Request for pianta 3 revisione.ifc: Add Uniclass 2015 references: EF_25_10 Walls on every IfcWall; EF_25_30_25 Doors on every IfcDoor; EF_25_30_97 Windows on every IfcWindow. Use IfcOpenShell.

First a look at what the model holds.

```python
import ifcopenshell

model = ifcopenshell.open("pianta 3 revisione.ifc")
print(model.schema)
print("classifications:", [c.Name for c in model.by_type("IfcClassification")])
for ifc_class in ("IfcDoor", "IfcRoof", "IfcStair", "IfcWall", "IfcWindow"):
    print(ifc_class, len(model.by_type(ifc_class)))
```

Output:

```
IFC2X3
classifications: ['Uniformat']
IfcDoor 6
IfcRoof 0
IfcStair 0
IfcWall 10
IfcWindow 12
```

```python
import ifcopenshell
import ifcopenshell.api.classification

model = ifcopenshell.open("pianta 3 revisione.ifc")

# IFC2X3 requires Source and Edition and has no link from the project to the system.
system = model.create_entity("IfcClassification", Source="NBS", Edition="2015", Name="Uniclass 2015")

codes = {
    "IfcWall": ("EF_25_10", "Walls"),
    "IfcDoor": ("EF_25_30_25", "Doors"),
    "IfcWindow": ("EF_25_30_97", "Windows"),
}
for ifc_class, (code, name) in codes.items():
    products = model.by_type(ifc_class)
    ifcopenshell.api.classification.add_reference(
        model, products=products, classification=system, identification=code, name=name
    )
    print(code, len(products))

model.write("pianta 3 revisione-out.ifc")
```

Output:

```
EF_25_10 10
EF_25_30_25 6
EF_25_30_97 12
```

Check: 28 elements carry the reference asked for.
